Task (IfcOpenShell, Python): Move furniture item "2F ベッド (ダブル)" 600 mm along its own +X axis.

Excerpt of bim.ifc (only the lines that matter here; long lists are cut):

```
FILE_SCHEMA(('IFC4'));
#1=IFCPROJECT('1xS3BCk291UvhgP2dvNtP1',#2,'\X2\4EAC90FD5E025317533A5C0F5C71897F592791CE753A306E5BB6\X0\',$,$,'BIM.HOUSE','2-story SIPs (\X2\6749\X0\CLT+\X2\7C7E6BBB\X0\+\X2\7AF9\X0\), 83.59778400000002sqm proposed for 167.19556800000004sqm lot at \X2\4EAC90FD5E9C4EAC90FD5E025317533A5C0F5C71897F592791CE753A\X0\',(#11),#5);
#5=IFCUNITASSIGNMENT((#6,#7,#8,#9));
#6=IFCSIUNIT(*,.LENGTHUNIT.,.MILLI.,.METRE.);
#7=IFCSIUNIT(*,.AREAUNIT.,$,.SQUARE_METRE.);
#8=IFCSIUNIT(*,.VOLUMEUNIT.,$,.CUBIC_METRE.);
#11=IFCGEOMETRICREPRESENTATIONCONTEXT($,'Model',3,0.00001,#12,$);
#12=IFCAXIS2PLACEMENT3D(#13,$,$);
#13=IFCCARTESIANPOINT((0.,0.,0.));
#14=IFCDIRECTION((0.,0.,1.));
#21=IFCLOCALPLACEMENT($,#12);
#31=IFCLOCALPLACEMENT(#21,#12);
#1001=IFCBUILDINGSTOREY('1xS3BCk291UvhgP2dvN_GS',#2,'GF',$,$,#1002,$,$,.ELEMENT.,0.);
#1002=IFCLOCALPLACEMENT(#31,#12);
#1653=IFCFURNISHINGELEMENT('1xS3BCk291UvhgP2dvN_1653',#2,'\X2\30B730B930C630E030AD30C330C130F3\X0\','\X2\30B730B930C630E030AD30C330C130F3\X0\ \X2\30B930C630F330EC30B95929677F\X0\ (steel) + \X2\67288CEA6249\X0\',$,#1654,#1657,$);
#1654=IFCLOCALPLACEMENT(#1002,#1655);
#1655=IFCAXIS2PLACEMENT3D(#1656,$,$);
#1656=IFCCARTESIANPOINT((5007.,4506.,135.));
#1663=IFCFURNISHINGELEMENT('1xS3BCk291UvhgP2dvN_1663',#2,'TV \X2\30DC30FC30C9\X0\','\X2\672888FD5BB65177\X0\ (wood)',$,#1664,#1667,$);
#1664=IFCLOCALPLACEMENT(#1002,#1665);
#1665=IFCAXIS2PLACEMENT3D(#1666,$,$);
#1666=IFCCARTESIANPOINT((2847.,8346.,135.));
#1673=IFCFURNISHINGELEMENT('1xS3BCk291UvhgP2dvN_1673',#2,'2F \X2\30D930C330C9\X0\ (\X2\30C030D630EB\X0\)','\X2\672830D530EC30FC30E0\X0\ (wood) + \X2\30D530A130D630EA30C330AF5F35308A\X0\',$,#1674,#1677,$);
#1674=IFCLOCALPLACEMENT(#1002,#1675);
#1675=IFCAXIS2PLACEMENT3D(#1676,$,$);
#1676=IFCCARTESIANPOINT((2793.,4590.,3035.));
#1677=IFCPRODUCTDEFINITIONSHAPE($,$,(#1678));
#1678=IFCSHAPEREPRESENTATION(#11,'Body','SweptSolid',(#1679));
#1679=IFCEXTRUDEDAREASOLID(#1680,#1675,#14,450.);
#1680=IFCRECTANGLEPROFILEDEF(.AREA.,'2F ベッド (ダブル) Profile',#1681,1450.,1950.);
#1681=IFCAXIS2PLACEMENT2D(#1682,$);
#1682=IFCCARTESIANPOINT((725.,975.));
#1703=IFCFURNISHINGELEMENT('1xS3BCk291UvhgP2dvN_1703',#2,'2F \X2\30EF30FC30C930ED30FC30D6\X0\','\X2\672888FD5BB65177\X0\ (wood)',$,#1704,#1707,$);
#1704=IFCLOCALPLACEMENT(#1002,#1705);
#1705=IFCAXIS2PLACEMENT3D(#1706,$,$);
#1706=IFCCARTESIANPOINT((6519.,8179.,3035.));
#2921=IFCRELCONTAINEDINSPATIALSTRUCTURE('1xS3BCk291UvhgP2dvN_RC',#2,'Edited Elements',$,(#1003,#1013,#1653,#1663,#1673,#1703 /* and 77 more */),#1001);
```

```python
import ifcopenshell
import ifcopenshell.api.geometry
import ifcopenshell.util.placement
import ifcopenshell.util.unit

model = ifcopenshell.open("bim.ifc")
unit_scale = ifcopenshell.util.unit.calculate_unit_scale(model)

item = model.by_id(1673)
matrix = ifcopenshell.util.placement.get_local_placement(item.ObjectPlacement)
matrix[:3, 3] += matrix[:3, 0] * 0.6 / unit_scale
ifcopenshell.api.geometry.edit_object_placement(model, product=item, matrix=matrix, is_si=False)

print(ifcopenshell.util.placement.get_local_placement(item.ObjectPlacement).round(3) + 0.0)

model.write("bim-out.ifc")
```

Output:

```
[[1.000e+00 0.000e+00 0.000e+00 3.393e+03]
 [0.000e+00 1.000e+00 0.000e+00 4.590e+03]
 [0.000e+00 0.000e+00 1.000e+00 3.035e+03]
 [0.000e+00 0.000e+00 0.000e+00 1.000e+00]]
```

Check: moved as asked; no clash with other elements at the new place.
